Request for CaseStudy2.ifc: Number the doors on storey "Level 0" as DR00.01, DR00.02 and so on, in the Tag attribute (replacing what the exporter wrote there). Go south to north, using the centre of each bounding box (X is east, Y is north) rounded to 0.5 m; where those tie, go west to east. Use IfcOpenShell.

First a look at what the model holds.

```python
import ifcopenshell
import ifcopenshell.util.element
import ifcopenshell.util.placement

model = ifcopenshell.open("CaseStudy2.ifc")
print(model.schema)
storey = next(s for s in model.by_type("IfcBuildingStorey") if s.Name == "Level 0")
doors = [e for e in ifcopenshell.util.element.get_decomposition(storey) if e.is_a("IfcDoor")]
for e in sorted(doors, key=lambda e: e.id()):
    origin = ifcopenshell.util.placement.get_local_placement(e.ObjectPlacement)[:3, 3]
    print(e.id(), e.Tag, e.Name, origin.round(2) + 0.0, sep=" | ")
```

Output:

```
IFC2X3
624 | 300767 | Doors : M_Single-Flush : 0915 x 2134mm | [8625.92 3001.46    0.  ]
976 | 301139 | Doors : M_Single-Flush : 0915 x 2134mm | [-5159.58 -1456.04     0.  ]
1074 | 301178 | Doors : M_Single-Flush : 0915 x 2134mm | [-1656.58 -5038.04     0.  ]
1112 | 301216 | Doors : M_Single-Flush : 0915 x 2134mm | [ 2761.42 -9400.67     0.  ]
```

```python
import ifcopenshell
import ifcopenshell.geom
import ifcopenshell.util.element
import ifcopenshell.util.shape

model = ifcopenshell.open("CaseStudy2.ifc")
settings = ifcopenshell.geom.settings()
settings.set("use-world-coords", True)


def centre(element):
    shape = ifcopenshell.geom.create_shape(settings, element)
    return ifcopenshell.util.shape.get_bbox_centroid(shape.geometry)


storey = next(s for s in model.by_type("IfcBuildingStorey") if s.Name == "Level 0")
doors = [e for e in ifcopenshell.util.element.get_decomposition(storey) if e.is_a("IfcDoor")]

# Insertion points can sit at a corner or the storey origin, so sort by the geometry (in metres).
centres = {e: centre(e) for e in doors}
doors.sort(key=lambda e: (round(centres[e][1] / 0.5), centres[e][0]))

for i, e in enumerate(doors, start=1):
    number = f"DR00.{i:02d}"
    e.Tag = number
    print(e.id(), number)

model.write("CaseStudy2_updated.ifc")
```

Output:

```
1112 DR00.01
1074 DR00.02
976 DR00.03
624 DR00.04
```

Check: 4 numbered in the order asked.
